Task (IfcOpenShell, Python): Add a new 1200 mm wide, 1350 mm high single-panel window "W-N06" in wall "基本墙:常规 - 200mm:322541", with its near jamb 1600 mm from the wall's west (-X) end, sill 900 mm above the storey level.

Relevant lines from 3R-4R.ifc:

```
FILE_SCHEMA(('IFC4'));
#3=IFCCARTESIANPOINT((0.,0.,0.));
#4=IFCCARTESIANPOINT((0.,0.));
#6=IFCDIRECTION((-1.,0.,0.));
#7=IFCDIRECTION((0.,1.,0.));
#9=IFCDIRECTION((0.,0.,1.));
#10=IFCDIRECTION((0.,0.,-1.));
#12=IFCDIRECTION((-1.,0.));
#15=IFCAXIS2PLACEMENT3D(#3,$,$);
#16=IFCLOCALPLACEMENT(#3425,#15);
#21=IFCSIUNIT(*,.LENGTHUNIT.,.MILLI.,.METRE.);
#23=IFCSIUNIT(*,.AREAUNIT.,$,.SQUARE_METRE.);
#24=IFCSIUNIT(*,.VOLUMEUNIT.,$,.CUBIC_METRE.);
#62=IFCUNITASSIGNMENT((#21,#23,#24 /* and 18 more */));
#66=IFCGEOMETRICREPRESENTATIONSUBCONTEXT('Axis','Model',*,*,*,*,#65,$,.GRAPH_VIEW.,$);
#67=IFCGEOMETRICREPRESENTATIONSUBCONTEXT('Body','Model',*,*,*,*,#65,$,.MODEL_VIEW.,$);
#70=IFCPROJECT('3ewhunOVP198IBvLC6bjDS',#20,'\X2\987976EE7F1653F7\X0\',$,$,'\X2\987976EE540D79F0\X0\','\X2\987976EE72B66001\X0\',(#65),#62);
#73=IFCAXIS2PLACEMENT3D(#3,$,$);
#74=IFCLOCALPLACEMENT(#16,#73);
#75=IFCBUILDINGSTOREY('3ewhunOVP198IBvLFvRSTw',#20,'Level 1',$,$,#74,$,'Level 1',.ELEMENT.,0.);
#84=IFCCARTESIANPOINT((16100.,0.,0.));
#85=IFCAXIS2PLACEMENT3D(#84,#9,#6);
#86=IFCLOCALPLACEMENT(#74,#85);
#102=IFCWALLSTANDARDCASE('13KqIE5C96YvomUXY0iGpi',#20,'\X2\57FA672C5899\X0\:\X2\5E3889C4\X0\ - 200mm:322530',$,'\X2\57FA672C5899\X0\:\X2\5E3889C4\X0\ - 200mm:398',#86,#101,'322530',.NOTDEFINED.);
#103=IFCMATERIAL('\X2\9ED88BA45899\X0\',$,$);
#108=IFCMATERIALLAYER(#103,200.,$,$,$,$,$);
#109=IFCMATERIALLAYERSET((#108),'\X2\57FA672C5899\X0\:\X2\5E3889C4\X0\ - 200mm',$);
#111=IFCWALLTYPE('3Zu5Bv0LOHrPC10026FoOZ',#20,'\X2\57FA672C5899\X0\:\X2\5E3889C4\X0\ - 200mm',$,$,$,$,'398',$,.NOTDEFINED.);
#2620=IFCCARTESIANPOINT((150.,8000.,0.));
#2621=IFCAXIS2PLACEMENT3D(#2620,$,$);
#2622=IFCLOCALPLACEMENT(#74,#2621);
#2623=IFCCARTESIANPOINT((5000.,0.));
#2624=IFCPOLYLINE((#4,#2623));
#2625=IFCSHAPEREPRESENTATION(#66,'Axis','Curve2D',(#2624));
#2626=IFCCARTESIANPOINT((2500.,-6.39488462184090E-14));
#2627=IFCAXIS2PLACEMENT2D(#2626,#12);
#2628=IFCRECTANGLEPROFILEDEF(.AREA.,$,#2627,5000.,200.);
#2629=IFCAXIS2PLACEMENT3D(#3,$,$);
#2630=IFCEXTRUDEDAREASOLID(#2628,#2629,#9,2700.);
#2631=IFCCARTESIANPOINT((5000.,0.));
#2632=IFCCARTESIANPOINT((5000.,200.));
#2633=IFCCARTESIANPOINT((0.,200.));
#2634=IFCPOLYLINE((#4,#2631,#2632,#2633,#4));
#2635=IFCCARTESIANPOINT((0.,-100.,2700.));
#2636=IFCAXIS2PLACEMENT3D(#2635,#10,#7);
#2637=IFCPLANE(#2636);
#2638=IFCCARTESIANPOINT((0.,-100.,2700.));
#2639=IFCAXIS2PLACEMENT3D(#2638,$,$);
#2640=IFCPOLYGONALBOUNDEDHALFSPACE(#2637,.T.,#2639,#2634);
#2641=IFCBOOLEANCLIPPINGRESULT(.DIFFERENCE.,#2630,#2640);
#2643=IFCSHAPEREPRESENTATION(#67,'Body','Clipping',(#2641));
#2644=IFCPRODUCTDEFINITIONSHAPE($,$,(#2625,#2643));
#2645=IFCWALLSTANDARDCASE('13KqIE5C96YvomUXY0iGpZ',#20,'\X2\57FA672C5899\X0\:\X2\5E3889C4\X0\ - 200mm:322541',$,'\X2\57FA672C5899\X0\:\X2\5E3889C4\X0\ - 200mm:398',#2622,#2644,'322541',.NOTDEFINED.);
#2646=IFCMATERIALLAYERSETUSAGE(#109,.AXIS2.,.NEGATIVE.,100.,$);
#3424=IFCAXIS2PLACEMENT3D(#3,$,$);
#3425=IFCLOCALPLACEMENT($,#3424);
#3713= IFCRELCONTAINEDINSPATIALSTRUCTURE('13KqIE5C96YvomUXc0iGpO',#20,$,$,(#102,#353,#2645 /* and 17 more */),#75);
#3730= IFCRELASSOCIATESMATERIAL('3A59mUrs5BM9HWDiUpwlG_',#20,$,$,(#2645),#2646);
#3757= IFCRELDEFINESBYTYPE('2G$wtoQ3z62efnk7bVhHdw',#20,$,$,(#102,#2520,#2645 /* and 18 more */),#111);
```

```python
import numpy as np
import ifcopenshell
import ifcopenshell.api.feature
import ifcopenshell.api.geometry
import ifcopenshell.api.root
import ifcopenshell.api.spatial
import ifcopenshell.geom
import ifcopenshell.util.element
import ifcopenshell.util.placement
import ifcopenshell.util.representation
import ifcopenshell.util.shape
import ifcopenshell.util.unit

model = ifcopenshell.open("3R-4R.ifc")
unit_scale = ifcopenshell.util.unit.calculate_unit_scale(model)
settings = ifcopenshell.geom.settings()


def volume(element):
    """Net volume in cubic metres, openings subtracted."""
    shape = ifcopenshell.geom.create_shape(settings, element)
    return ifcopenshell.util.shape.get_volume(shape.geometry)


wall = model.by_guid("13KqIE5C96YvomUXY0iGpZ")
storey = ifcopenshell.util.element.get_container(wall, ifc_class="IfcBuildingStorey")
context = ifcopenshell.util.representation.get_context(model, "Model", "Body", "MODEL_VIEW")
before = volume(wall)

width, height, from_end, sill = 1.2, 1.35, 1.6, 0.9  # metres

# The wall runs along its own X axis, and the end named is its -X end.
wall_shape = ifcopenshell.geom.create_shape(settings, wall)
x, y, z = ifcopenshell.util.shape.get_vertices(wall_shape.geometry).T
start = x.min() + from_end
face, thickness = float(y.min()), float(y.max() - y.min())
wall_matrix = ifcopenshell.util.placement.get_local_placement(wall.ObjectPlacement)
level = ifcopenshell.util.placement.get_local_placement(storey.ObjectPlacement)[2, 3]


def in_wall(x, y):
    """Placement at x, y metres in the wall's axes, at sill height."""
    matrix = wall_matrix.copy()
    matrix[:, 3] = wall_matrix @ np.array([x / unit_scale, y / unit_scale, 0.0, 1.0])
    matrix[2, 3] = level + sill / unit_scale
    return matrix


# Opening: a box that overshoots both wall faces by 50 mm.
opening = ifcopenshell.api.root.create_entity(model, ifc_class="IfcOpeningElement", predefined_type="OPENING")
box = ifcopenshell.api.geometry.add_wall_representation(
    model, context=context, length=width, height=height, thickness=thickness + 0.1
)
ifcopenshell.api.geometry.assign_representation(model, product=opening, representation=box)
ifcopenshell.api.geometry.edit_object_placement(model, product=opening, matrix=in_wall(start, face - 0.05), is_si=False)
ifcopenshell.api.feature.add_feature(model, feature=opening, element=wall)

window = ifcopenshell.api.root.create_entity(model, ifc_class="IfcWindow", name="W-N06", predefined_type="WINDOW")
window.OverallWidth, window.OverallHeight = width / unit_scale, height / unit_scale
window.PartitioningType = "SINGLE_PANEL"
body = ifcopenshell.api.geometry.add_window_representation(
    model,
    context=context,
    overall_width=window.OverallWidth,
    overall_height=window.OverallHeight,
    partition_type="SINGLE_PANEL",
)
ifcopenshell.api.geometry.assign_representation(model, product=window, representation=body)
ifcopenshell.api.spatial.assign_container(model, products=[window], relating_structure=storey)
ifcopenshell.api.feature.add_filling(model, opening=opening, element=window)

# Centre the window in the wall's thickness.
ifcopenshell.api.geometry.edit_object_placement(model, product=window, matrix=in_wall(start, face), is_si=False)
window_shape = ifcopenshell.geom.create_shape(settings, window)
depth = ifcopenshell.util.shape.get_vertices(window_shape.geometry)[:, 1]
offset = face + thickness / 2 - (depth.min() + depth.max()) / 2
ifcopenshell.api.geometry.edit_object_placement(model, product=window, matrix=in_wall(start, offset), is_si=False)

after = volume(wall)

print(f"wall volume {before:.3f} -> {after:.3f} m3")

model.write("3R-4R_rev.ifc")
```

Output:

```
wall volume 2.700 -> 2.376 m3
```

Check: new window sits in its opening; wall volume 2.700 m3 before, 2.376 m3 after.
